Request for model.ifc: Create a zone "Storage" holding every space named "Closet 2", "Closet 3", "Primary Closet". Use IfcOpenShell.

First a look at what the model holds.

```python
import ifcopenshell

model = ifcopenshell.open("model.ifc")
print(model.schema)
seen = {}
for space in model.by_type("IfcSpace"):
    seen[space.LongName] = seen.get(space.LongName, 0) + 1
for name, count in sorted(seen.items(), key=str):
    print(count, "x", name)
print("zones:", [z.Name for z in model.by_type("IfcZone")][:20])
```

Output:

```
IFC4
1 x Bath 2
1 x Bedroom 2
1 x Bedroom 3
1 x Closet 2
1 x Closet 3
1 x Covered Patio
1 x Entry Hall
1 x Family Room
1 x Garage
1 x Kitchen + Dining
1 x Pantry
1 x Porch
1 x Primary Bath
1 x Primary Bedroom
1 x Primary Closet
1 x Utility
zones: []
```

```python
import ifcopenshell
import ifcopenshell.api.group
import ifcopenshell.api.root

model = ifcopenshell.open("model.ifc")

names = {"Closet 2", "Closet 3", "Primary Closet"}
spaces = [s for s in model.by_type("IfcSpace") if s.LongName in names]

zone = ifcopenshell.api.root.create_entity(model, ifc_class="IfcZone", name="Storage")
ifcopenshell.api.group.assign_group(model, products=spaces, group=zone)
print(len(spaces), "spaces in", zone.Name)

model.write("model_edited.ifc")
```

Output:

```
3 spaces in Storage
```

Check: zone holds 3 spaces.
